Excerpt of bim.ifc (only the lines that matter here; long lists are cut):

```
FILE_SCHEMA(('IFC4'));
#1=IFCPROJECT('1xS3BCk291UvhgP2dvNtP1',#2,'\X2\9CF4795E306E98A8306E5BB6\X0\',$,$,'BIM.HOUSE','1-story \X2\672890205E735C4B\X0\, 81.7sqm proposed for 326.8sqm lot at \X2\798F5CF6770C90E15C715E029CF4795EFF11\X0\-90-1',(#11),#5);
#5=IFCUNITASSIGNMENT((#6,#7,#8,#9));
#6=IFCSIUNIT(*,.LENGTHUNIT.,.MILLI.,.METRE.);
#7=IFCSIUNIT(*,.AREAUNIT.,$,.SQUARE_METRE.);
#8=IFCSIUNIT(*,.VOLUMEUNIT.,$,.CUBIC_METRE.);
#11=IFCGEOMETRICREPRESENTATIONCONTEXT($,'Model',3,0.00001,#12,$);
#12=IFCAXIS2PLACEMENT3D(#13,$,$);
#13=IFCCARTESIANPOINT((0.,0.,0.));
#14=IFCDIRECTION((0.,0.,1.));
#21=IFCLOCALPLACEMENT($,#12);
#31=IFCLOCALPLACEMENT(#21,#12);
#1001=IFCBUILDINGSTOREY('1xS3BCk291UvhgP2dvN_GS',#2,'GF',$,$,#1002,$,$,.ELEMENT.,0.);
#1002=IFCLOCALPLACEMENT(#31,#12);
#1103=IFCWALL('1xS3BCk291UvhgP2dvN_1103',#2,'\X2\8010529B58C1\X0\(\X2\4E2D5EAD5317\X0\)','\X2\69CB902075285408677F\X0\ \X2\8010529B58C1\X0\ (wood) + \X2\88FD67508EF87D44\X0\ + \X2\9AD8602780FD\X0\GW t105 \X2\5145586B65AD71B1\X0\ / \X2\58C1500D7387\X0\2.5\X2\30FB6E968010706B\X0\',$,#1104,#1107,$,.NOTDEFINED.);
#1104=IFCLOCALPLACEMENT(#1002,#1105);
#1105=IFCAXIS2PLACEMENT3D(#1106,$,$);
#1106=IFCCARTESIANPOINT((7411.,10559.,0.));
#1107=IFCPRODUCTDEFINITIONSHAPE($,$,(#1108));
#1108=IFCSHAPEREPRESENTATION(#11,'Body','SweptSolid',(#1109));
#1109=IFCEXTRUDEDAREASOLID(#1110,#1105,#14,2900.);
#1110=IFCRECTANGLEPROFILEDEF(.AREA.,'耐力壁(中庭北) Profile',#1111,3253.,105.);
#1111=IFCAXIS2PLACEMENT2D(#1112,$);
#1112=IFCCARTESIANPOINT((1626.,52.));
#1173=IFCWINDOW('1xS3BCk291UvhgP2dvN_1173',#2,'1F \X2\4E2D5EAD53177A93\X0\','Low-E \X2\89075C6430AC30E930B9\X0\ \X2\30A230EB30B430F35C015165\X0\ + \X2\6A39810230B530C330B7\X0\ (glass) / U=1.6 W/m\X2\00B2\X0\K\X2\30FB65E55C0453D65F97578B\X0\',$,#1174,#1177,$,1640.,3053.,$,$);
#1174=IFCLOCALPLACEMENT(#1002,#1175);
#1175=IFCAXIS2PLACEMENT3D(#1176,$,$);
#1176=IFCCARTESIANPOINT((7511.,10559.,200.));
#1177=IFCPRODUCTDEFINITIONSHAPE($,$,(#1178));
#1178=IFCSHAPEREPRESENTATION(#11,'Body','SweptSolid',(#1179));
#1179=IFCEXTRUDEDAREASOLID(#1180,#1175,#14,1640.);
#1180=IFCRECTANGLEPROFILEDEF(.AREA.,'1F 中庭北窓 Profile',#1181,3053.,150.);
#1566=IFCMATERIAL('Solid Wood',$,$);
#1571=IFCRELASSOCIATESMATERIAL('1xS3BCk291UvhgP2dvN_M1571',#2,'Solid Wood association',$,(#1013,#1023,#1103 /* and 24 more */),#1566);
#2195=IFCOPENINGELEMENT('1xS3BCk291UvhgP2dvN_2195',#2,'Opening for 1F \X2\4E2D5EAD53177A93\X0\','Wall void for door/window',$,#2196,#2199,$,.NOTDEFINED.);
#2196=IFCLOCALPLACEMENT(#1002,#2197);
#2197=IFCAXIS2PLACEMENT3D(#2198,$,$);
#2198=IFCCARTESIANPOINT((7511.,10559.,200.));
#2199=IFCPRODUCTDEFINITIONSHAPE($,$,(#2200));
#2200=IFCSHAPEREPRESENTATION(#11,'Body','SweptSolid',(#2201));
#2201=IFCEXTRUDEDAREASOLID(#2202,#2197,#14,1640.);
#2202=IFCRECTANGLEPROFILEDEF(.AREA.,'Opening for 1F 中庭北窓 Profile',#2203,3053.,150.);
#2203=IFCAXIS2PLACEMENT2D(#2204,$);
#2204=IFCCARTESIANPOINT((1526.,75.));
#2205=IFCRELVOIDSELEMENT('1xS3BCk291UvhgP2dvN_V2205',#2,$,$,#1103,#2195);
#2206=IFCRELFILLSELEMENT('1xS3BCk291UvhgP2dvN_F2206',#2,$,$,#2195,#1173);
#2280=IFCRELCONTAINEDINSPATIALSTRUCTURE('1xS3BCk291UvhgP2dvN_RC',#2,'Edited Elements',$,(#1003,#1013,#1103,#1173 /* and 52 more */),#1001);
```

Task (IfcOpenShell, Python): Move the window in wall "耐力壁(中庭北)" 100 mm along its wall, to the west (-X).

```python
import ifcopenshell
import ifcopenshell.api.geometry
import ifcopenshell.util.placement
import ifcopenshell.util.unit

model = ifcopenshell.open("bim.ifc")
unit_scale = ifcopenshell.util.unit.calculate_unit_scale(model)

window = model.by_id(1173)
opening = window.FillsVoids[0].RelatingOpeningElement
wall = opening.VoidsElements[0].RelatingBuildingElement

wall_matrix = ifcopenshell.util.placement.get_local_placement(wall.ObjectPlacement)
shift = wall_matrix[:3, 0] * -0.1 / unit_scale
before = ifcopenshell.util.placement.get_local_placement(window.ObjectPlacement)[:3, 3].copy()

# The window is not placed relative to its opening, so move both.
for product in (opening, window):
    matrix = ifcopenshell.util.placement.get_local_placement(product.ObjectPlacement)
    matrix[:3, 3] += shift
    ifcopenshell.api.geometry.edit_object_placement(model, product=product, matrix=matrix, is_si=False)

after = ifcopenshell.util.placement.get_local_placement(window.ObjectPlacement)[:3, 3]
print("window moved by", (after - before).round(3) + 0.0)

model.write("bim_updated.ifc")
```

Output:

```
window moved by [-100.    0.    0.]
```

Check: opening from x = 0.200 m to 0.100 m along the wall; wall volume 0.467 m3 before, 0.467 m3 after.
